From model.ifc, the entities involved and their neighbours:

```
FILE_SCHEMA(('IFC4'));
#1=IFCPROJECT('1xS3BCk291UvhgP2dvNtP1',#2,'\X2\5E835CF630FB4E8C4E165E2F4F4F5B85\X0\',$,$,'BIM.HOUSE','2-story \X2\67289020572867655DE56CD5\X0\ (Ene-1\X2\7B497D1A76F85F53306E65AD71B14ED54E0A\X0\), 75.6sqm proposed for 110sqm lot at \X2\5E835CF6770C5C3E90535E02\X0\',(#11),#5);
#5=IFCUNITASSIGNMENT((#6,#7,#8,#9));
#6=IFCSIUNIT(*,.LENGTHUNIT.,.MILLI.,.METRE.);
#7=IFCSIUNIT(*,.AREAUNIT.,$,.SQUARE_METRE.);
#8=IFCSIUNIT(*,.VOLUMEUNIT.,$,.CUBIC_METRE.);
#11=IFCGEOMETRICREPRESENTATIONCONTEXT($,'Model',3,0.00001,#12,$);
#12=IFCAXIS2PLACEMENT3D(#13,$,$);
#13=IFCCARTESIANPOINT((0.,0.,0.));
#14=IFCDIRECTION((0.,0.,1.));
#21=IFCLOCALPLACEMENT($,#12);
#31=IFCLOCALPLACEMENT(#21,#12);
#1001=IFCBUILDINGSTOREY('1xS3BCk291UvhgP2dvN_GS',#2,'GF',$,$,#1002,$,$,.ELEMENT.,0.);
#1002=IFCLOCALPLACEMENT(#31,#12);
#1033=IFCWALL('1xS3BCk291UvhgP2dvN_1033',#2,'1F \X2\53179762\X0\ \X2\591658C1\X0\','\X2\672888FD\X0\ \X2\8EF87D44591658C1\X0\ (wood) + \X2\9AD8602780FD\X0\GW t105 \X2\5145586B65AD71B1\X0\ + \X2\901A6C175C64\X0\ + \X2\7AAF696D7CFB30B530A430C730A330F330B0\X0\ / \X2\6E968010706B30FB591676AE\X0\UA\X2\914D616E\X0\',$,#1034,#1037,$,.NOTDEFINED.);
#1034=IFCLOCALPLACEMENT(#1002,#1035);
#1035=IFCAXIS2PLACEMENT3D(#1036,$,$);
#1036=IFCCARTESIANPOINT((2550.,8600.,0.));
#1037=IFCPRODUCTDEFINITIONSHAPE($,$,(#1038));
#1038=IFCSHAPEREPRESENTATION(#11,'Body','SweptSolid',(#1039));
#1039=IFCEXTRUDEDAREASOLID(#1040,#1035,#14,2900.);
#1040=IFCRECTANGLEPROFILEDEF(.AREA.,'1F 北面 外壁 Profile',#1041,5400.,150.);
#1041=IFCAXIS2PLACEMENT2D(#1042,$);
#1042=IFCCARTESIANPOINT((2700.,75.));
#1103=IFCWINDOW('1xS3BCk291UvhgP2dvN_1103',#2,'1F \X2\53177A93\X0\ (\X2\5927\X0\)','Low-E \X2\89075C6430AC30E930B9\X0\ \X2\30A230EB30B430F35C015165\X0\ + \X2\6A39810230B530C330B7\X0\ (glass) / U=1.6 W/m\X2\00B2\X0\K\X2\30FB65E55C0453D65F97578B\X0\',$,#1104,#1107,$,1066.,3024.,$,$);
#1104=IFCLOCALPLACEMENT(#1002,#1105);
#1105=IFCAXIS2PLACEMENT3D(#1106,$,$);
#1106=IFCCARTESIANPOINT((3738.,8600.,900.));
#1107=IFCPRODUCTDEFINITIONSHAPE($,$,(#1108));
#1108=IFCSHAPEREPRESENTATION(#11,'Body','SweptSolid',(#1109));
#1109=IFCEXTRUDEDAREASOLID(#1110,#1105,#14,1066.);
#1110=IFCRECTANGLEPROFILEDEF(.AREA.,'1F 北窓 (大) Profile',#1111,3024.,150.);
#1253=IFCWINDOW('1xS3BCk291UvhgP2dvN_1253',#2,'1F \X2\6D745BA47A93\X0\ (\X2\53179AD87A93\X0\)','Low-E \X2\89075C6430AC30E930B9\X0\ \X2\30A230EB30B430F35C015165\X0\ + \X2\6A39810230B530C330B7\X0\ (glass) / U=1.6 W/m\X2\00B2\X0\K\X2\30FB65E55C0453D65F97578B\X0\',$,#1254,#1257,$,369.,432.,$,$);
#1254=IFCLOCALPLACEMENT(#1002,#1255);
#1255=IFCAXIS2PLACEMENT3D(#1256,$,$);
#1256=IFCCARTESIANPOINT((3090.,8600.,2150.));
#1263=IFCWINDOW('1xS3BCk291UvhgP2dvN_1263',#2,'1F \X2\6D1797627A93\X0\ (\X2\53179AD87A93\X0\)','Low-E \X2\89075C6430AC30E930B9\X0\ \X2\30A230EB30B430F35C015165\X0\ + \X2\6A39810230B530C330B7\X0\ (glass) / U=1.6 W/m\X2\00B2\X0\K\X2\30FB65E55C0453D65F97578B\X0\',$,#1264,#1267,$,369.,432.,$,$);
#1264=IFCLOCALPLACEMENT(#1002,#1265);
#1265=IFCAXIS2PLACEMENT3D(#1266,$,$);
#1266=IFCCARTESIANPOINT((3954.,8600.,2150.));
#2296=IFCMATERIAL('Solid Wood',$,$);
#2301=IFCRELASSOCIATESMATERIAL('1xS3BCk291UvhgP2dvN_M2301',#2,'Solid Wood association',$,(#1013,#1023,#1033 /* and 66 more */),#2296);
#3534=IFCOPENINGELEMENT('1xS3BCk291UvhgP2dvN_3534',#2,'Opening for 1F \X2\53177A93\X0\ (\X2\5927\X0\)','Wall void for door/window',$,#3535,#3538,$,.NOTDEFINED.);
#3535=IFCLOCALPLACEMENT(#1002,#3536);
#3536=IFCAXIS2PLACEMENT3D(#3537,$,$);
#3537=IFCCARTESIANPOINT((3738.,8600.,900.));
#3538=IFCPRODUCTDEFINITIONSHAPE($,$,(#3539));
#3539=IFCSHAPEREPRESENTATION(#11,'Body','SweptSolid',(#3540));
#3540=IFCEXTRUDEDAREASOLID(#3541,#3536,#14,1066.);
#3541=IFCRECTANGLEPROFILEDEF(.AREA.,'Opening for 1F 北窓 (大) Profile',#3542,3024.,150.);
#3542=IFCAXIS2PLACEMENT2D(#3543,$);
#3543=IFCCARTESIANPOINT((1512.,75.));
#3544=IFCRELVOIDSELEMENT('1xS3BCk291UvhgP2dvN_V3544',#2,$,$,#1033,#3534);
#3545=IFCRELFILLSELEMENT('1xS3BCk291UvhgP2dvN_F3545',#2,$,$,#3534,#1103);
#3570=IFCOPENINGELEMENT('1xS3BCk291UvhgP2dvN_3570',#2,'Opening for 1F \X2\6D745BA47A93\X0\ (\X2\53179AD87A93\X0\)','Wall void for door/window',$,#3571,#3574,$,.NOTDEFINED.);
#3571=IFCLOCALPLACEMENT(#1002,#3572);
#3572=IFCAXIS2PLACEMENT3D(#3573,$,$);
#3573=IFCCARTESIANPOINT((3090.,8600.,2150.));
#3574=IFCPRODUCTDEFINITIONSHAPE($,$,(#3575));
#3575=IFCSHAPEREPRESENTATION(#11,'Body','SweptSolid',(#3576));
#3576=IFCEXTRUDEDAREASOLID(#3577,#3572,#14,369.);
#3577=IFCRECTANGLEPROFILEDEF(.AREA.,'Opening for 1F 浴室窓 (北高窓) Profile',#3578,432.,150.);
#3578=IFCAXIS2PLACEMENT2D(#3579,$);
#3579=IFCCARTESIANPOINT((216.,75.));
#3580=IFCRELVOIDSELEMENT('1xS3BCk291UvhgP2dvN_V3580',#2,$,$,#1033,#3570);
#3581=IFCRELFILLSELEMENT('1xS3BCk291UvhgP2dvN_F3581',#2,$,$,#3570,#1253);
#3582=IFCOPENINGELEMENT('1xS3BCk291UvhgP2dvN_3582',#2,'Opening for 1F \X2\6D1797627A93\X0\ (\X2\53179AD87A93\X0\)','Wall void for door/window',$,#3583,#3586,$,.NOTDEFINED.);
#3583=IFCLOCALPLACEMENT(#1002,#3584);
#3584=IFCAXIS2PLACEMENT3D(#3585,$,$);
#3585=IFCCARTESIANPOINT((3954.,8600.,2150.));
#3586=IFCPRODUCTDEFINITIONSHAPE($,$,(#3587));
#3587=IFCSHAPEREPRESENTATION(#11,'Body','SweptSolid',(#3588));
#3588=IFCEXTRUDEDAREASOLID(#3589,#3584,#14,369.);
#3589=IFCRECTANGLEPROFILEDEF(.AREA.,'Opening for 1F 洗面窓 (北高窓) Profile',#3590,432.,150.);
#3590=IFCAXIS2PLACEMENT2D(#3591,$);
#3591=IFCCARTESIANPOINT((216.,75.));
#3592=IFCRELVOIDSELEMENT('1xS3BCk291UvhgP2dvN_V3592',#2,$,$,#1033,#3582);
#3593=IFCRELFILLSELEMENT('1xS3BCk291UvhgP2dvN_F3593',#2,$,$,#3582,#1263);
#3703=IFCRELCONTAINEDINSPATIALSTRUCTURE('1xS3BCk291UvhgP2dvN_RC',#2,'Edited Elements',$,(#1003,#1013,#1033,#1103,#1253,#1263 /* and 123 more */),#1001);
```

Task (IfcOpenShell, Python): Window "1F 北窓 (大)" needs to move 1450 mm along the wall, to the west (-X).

```python
import ifcopenshell
import ifcopenshell.api.geometry
import ifcopenshell.util.placement

model = ifcopenshell.open("model.ifc")

window = model.by_id(1103)
opening = window.FillsVoids[0].RelatingOpeningElement
wall = opening.VoidsElements[0].RelatingBuildingElement

wall_matrix = ifcopenshell.util.placement.get_local_placement(wall.ObjectPlacement)
shift = wall_matrix[:3, 0] * -1450.0
before = ifcopenshell.util.placement.get_local_placement(window.ObjectPlacement)[:3, 3].copy()

# The window is not placed relative to its opening, so move both.
for product in (opening, window):
    matrix = ifcopenshell.util.placement.get_local_placement(product.ObjectPlacement)
    matrix[:3, 3] += shift
    ifcopenshell.api.geometry.edit_object_placement(model, product=product, matrix=matrix, is_si=False)

after = ifcopenshell.util.placement.get_local_placement(window.ObjectPlacement)[:3, 3]
print("window moved by", (after - before).round(3) + 0.0)

model.write("model_edited.ifc")
```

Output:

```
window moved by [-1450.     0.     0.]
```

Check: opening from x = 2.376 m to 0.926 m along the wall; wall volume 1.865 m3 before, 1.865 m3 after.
